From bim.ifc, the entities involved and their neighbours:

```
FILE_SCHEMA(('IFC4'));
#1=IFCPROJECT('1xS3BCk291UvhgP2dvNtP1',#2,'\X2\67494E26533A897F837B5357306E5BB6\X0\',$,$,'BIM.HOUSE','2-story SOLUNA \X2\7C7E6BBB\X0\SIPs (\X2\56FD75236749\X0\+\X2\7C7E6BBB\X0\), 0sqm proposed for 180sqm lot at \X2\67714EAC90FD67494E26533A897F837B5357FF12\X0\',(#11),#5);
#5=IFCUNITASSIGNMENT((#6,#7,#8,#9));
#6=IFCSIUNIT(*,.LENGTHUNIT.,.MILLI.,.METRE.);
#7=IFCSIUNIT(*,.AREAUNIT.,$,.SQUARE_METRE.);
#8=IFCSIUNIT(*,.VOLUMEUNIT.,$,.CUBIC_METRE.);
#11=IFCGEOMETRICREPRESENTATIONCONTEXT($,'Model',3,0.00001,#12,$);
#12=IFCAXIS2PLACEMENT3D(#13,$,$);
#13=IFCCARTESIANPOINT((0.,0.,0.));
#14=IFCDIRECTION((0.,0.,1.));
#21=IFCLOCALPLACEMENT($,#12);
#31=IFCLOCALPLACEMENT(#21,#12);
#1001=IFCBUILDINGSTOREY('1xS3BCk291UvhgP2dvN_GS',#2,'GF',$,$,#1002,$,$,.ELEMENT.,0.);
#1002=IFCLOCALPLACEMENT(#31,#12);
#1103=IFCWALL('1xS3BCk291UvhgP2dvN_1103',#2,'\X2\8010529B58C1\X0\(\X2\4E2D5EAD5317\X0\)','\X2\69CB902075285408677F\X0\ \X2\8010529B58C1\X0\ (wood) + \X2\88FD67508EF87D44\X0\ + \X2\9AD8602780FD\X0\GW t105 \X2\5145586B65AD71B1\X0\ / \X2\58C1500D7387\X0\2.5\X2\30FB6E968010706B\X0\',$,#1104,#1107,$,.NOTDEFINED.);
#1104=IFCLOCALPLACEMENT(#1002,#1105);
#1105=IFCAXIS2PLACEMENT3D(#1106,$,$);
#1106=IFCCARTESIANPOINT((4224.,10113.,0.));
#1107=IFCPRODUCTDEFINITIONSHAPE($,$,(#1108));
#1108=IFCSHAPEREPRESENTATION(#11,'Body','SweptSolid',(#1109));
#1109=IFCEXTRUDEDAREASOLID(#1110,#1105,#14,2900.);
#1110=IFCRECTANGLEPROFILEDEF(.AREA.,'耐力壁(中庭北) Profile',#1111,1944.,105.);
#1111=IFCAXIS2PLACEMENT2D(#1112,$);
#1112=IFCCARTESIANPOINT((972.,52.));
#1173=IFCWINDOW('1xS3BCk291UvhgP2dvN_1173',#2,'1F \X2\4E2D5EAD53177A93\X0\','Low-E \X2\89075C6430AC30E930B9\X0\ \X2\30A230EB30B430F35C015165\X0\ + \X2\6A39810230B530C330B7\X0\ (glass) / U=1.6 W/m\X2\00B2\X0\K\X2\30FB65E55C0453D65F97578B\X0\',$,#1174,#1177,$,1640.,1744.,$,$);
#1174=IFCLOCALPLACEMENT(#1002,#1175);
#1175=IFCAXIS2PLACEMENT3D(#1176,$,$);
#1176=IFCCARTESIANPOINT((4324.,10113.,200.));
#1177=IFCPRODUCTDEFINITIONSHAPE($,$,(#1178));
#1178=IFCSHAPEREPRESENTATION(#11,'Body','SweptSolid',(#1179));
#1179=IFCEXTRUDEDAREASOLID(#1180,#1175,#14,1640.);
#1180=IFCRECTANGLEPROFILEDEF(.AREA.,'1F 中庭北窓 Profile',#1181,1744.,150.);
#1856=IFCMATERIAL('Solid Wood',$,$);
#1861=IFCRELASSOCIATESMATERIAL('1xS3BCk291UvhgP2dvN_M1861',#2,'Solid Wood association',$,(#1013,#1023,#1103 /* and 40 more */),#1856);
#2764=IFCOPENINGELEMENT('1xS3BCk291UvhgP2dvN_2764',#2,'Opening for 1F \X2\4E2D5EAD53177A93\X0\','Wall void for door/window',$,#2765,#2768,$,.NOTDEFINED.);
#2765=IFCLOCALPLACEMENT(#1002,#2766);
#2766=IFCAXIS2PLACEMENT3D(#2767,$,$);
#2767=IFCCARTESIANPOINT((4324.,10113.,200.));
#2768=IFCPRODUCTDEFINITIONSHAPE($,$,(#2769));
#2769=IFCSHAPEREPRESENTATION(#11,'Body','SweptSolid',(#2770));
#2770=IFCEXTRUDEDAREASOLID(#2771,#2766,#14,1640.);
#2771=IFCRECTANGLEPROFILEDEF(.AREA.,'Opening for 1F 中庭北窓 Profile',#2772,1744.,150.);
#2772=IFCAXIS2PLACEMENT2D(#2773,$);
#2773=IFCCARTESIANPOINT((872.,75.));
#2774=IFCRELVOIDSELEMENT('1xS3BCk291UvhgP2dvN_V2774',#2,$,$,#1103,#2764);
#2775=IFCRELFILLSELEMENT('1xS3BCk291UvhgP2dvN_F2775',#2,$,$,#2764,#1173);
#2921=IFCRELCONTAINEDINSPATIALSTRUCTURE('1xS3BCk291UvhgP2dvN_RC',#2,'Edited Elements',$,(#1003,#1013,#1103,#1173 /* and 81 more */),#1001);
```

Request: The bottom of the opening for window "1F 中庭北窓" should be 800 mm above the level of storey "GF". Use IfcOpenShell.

```python
import numpy as np
import ifcopenshell
import ifcopenshell.api.geometry
import ifcopenshell.geom
import ifcopenshell.util.element
import ifcopenshell.util.placement
import ifcopenshell.util.shape
import ifcopenshell.util.unit

model = ifcopenshell.open("bim.ifc")
unit_scale = ifcopenshell.util.unit.calculate_unit_scale(model)

window = model.by_guid("1xS3BCk291UvhgP2dvN_1173")
opening = window.FillsVoids[0].RelatingOpeningElement
storey = ifcopenshell.util.element.get_container(window, ifc_class="IfcBuildingStorey")
level = ifcopenshell.util.placement.get_local_placement(storey.ObjectPlacement)[2, 3]

# The opening's origin need not be at the sill, so measure its lowest point.
shape = ifcopenshell.geom.create_shape(ifcopenshell.geom.settings(), opening)
bottom = ifcopenshell.util.shape.get_shape_bottom_elevation(shape, shape.geometry) / unit_scale
dz = level + 800.0 - bottom

shift = np.array([0.0, 0.0, dz])
# The window is not placed relative to its opening, so move both.
for product in (opening, window):
    matrix = ifcopenshell.util.placement.get_local_placement(product.ObjectPlacement)
    matrix[:3, 3] += shift
    ifcopenshell.api.geometry.edit_object_placement(model, product=product, matrix=matrix, is_si=False)

print(f"moved by {dz * unit_scale:+.3f} m")

model.write("bim_updated.ifc")
```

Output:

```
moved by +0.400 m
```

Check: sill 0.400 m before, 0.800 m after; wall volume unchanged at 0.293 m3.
